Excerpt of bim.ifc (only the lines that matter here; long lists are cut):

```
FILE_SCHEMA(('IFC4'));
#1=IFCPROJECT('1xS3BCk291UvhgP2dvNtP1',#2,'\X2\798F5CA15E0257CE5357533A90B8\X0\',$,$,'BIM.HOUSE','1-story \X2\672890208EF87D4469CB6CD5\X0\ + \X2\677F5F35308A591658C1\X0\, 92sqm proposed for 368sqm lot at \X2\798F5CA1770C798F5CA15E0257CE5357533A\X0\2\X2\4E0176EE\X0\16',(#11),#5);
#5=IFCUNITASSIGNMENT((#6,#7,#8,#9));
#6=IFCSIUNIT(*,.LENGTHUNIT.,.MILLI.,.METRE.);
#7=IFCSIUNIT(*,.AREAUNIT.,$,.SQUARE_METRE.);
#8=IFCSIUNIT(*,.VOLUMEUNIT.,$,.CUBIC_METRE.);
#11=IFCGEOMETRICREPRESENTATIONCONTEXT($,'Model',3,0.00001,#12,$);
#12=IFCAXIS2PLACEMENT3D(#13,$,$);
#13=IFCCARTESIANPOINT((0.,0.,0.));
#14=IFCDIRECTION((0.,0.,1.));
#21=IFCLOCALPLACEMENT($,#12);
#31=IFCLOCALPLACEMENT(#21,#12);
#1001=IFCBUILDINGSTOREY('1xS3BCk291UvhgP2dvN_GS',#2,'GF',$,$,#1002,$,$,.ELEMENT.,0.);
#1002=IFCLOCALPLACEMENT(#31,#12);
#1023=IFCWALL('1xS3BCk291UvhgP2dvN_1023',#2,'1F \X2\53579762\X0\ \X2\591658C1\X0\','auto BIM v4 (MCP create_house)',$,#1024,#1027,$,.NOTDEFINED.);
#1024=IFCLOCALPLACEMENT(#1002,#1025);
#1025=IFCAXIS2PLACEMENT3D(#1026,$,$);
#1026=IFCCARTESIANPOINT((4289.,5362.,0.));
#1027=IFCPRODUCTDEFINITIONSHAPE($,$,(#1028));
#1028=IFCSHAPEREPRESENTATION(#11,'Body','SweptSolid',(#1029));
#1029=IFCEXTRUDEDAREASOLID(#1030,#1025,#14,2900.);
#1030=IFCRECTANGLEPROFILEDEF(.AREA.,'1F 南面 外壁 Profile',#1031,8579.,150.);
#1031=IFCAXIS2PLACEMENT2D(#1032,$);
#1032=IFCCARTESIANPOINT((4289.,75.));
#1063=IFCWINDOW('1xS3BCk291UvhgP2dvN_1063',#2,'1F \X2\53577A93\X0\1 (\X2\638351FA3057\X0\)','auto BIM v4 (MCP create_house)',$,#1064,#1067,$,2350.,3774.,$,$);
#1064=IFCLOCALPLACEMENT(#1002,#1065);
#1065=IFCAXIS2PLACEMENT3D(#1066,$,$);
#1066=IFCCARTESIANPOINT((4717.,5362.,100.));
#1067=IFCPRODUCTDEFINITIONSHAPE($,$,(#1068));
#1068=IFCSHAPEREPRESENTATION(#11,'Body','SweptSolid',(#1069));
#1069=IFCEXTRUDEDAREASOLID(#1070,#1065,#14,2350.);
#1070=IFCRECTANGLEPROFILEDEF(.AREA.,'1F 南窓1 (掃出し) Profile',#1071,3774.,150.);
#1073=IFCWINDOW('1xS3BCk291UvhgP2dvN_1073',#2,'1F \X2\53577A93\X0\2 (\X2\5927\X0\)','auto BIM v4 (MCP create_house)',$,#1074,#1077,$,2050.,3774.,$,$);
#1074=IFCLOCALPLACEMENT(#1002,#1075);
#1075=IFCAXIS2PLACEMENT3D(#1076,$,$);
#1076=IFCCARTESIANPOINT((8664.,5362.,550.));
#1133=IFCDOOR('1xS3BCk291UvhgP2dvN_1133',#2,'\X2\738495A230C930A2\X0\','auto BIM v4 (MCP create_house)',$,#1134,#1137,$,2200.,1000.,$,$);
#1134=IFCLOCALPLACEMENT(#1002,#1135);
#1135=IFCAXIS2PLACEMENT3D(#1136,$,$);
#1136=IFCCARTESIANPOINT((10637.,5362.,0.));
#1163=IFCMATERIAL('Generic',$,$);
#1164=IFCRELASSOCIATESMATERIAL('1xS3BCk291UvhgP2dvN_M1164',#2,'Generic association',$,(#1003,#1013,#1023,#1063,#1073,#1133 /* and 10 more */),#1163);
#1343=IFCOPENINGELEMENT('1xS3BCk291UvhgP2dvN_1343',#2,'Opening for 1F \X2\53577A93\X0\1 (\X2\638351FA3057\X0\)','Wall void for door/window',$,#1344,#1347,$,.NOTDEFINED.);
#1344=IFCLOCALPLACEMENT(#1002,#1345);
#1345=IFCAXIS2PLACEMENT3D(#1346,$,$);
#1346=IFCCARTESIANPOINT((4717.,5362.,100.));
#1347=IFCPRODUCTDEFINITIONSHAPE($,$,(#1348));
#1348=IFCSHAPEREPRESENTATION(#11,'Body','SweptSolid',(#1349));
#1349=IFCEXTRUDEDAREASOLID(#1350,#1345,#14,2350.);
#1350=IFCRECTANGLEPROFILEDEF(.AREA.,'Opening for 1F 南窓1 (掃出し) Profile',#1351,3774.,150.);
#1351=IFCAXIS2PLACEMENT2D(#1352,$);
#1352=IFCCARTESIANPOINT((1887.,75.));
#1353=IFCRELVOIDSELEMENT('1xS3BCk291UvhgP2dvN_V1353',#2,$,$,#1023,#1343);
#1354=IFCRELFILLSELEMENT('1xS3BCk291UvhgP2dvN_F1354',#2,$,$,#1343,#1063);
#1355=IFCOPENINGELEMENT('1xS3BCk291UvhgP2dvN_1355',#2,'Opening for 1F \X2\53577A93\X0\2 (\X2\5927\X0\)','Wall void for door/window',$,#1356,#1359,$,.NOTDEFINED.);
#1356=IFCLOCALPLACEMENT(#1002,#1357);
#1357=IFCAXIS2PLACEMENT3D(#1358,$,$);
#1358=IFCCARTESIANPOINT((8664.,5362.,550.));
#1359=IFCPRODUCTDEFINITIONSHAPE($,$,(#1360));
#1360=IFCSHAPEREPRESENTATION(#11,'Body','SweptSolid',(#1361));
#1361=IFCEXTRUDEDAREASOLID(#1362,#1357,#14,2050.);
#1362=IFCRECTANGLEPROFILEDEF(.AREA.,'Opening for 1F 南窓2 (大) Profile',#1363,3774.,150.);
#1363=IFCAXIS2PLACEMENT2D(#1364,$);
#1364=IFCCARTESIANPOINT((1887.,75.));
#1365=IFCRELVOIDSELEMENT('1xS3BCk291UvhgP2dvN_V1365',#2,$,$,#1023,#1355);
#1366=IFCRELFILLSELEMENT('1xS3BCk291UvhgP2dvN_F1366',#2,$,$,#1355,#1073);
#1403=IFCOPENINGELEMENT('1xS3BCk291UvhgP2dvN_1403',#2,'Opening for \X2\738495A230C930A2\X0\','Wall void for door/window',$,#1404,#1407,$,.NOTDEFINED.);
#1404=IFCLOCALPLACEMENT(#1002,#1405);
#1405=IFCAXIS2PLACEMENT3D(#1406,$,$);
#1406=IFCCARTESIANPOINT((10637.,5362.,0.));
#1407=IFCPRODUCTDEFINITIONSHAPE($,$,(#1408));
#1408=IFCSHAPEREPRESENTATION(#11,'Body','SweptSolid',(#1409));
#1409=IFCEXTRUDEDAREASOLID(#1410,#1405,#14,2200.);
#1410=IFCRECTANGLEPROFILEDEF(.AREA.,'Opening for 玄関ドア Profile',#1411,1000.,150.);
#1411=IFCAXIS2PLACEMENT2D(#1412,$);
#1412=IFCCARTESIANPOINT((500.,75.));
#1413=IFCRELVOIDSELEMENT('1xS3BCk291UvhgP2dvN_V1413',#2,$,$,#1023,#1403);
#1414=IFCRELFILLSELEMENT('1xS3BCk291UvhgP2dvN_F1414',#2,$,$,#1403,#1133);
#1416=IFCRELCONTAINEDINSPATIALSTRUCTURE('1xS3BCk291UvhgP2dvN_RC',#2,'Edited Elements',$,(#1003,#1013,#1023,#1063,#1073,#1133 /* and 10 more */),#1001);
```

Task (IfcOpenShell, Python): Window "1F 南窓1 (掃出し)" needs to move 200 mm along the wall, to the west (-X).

```python
import ifcopenshell
import ifcopenshell.api.geometry
import ifcopenshell.util.placement

model = ifcopenshell.open("bim.ifc")

window = model.by_guid("1xS3BCk291UvhgP2dvN_1063")
opening = window.FillsVoids[0].RelatingOpeningElement
wall = opening.VoidsElements[0].RelatingBuildingElement

wall_matrix = ifcopenshell.util.placement.get_local_placement(wall.ObjectPlacement)
shift = wall_matrix[:3, 0] * -200.0
before = ifcopenshell.util.placement.get_local_placement(window.ObjectPlacement)[:3, 3].copy()

# The window is not placed relative to its opening, so move both.
for product in (opening, window):
    matrix = ifcopenshell.util.placement.get_local_placement(product.ObjectPlacement)
    matrix[:3, 3] += shift
    ifcopenshell.api.geometry.edit_object_placement(model, product=product, matrix=matrix, is_si=False)

after = ifcopenshell.util.placement.get_local_placement(window.ObjectPlacement)[:3, 3]
print("window moved by", (after - before).round(3) + 0.0)

model.write("bim_edited.ifc")
```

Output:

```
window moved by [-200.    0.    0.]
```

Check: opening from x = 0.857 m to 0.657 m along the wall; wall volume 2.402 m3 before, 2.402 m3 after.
